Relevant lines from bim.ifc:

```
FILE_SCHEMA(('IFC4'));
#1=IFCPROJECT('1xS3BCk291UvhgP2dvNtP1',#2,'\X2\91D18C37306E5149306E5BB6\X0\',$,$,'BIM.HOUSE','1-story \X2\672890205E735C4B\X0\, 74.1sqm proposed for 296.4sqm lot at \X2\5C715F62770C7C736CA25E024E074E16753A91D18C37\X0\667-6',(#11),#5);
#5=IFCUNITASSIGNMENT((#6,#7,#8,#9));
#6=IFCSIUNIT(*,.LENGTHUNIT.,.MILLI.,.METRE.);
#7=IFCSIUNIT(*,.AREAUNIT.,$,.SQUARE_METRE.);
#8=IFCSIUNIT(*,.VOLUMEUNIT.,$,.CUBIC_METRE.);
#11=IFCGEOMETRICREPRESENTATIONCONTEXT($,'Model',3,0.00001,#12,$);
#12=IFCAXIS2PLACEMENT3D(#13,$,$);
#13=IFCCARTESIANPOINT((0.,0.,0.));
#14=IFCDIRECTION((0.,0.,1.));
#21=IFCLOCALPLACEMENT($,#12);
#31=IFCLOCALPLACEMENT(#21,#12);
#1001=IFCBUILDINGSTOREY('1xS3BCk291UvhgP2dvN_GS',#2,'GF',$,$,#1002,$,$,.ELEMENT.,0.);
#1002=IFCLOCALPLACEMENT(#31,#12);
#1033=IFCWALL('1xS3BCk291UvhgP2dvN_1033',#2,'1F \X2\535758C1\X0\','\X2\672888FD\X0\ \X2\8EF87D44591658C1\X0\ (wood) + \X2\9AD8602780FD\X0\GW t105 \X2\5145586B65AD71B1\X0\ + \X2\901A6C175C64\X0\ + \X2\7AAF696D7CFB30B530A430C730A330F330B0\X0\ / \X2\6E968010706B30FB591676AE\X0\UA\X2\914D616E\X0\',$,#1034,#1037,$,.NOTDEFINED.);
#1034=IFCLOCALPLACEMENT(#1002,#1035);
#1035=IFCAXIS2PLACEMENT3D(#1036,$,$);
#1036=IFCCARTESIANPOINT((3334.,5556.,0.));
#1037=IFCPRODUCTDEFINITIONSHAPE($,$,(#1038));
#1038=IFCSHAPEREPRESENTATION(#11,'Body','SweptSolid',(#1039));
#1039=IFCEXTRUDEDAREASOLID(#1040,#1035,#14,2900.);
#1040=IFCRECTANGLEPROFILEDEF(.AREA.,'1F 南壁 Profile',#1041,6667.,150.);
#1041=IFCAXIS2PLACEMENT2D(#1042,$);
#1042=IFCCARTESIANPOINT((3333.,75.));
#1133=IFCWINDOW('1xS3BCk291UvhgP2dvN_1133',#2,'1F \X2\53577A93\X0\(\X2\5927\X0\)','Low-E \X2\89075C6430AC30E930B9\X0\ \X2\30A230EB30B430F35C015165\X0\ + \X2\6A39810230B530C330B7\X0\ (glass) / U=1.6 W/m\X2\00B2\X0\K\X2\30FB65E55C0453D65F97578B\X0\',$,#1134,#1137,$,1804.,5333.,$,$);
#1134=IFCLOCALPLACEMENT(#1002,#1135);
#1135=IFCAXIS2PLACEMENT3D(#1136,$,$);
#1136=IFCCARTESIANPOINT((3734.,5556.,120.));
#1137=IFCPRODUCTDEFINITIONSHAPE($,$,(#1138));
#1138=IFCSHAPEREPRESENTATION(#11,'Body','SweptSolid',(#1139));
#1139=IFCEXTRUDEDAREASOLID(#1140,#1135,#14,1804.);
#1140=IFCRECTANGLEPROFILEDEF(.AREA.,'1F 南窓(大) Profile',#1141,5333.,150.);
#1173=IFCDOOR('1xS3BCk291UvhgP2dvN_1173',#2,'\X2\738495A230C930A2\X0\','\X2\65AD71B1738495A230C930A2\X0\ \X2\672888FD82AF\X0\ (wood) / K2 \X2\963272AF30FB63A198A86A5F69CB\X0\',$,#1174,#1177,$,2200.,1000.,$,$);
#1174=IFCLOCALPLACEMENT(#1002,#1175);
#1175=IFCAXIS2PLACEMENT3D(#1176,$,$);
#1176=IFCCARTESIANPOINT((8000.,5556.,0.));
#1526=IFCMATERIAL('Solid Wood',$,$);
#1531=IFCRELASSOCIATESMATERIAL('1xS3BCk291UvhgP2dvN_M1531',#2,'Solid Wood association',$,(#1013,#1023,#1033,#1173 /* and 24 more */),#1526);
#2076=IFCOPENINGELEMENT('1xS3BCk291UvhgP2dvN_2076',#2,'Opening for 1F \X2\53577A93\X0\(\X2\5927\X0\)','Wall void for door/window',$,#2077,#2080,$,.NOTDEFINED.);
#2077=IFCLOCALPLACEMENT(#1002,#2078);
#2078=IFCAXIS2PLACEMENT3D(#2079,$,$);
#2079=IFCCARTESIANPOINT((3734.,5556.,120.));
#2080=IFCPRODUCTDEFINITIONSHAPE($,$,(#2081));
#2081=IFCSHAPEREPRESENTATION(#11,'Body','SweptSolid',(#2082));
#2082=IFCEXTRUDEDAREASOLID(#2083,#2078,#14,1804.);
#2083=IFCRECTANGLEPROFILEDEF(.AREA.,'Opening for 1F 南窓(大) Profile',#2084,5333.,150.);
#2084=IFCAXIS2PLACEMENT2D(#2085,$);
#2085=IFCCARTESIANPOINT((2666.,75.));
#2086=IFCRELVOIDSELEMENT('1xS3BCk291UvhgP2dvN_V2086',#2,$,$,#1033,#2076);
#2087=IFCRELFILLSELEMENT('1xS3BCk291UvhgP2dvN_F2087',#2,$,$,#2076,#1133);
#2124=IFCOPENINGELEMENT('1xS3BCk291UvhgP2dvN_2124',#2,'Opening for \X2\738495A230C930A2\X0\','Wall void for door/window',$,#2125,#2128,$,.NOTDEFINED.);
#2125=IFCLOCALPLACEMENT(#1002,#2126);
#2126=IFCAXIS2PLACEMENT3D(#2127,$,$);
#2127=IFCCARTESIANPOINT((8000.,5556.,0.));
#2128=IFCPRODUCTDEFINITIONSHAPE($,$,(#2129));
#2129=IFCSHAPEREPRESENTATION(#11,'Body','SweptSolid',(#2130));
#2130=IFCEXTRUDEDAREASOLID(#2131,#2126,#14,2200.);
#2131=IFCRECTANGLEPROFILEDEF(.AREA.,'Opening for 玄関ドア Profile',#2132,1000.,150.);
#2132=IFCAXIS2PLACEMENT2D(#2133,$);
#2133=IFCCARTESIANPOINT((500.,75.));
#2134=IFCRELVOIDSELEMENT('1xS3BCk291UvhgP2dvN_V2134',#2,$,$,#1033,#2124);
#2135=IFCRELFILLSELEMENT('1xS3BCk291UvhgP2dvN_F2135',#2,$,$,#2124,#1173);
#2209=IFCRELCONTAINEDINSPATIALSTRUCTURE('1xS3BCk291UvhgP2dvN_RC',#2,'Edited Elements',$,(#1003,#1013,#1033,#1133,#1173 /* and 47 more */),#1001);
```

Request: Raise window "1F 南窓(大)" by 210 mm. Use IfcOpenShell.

```python
import numpy as np
import ifcopenshell
import ifcopenshell.api.geometry
import ifcopenshell.util.placement
import ifcopenshell.util.unit

model = ifcopenshell.open("bim.ifc")
unit_scale = ifcopenshell.util.unit.calculate_unit_scale(model)

window = model.by_id(1133)
opening = window.FillsVoids[0].RelatingOpeningElement
dz = 0.21 / unit_scale

shift = np.array([0.0, 0.0, dz])
# The window is not placed relative to its opening, so move both.
for product in (opening, window):
    matrix = ifcopenshell.util.placement.get_local_placement(product.ObjectPlacement)
    matrix[:3, 3] += shift
    ifcopenshell.api.geometry.edit_object_placement(model, product=product, matrix=matrix, is_si=False)

print(f"moved by {dz * unit_scale:+.3f} m")

model.write("bim-out.ifc")
```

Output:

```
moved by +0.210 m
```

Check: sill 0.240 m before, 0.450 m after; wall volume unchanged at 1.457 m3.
